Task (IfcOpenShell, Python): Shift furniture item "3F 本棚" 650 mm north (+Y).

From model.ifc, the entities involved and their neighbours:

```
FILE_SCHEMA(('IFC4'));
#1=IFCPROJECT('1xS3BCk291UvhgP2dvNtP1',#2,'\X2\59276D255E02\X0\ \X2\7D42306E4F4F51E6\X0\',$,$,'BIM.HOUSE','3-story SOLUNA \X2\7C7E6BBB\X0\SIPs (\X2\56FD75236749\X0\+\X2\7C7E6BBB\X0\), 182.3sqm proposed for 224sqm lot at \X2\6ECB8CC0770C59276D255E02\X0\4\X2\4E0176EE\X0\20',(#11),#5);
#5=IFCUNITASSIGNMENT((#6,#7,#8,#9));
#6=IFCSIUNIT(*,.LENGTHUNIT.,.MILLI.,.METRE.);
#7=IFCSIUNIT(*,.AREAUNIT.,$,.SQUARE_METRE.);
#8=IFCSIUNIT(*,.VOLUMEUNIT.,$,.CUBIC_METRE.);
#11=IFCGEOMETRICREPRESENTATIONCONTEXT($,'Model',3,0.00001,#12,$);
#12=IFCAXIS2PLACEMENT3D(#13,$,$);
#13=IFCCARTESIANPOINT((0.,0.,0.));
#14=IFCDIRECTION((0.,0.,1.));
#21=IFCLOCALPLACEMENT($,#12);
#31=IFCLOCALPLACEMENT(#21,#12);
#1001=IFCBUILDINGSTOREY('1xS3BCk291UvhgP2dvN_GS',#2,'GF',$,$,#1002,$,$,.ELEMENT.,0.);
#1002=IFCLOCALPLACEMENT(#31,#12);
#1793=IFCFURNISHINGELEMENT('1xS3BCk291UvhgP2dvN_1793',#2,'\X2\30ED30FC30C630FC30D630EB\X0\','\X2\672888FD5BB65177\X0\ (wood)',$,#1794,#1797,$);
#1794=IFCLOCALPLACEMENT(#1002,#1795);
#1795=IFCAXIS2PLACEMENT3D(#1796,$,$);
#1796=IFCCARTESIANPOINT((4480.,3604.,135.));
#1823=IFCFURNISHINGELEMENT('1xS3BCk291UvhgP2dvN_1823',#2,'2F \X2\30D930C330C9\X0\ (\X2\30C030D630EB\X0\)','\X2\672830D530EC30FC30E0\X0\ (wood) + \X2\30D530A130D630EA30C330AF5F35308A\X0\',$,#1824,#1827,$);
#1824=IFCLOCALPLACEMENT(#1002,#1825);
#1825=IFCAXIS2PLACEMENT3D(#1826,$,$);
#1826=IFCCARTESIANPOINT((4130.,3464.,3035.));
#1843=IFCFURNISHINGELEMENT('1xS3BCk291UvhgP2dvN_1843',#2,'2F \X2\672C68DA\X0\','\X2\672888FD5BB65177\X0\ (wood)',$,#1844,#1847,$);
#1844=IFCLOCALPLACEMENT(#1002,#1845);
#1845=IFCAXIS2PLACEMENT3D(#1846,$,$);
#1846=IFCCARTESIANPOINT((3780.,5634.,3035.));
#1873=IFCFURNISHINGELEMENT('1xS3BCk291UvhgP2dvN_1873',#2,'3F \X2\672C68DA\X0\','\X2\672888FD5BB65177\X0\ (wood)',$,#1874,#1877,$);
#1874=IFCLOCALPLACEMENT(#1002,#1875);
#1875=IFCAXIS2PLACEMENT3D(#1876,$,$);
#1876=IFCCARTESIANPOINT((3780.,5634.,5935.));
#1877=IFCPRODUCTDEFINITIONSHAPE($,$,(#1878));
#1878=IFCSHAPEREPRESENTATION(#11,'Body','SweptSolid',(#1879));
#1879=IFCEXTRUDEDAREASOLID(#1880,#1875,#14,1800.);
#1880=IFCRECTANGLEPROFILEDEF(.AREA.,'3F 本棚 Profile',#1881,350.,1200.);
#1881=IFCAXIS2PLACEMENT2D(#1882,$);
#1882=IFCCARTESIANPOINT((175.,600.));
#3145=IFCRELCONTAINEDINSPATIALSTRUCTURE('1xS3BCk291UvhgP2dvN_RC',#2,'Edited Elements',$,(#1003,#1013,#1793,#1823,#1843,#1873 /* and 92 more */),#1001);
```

```python
import ifcopenshell
import ifcopenshell.api.geometry
import ifcopenshell.util.placement

model = ifcopenshell.open("model.ifc")

item = model.by_guid("1xS3BCk291UvhgP2dvN_1873")
matrix = ifcopenshell.util.placement.get_local_placement(item.ObjectPlacement)
matrix[1, 3] += 650.0
ifcopenshell.api.geometry.edit_object_placement(model, product=item, matrix=matrix, is_si=False)

print(ifcopenshell.util.placement.get_local_placement(item.ObjectPlacement).round(3) + 0.0)

model.write("model_updated.ifc")
```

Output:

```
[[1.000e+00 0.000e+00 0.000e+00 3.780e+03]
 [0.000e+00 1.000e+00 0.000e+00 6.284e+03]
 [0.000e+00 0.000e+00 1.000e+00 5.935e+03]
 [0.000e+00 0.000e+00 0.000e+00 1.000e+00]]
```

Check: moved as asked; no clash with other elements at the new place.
